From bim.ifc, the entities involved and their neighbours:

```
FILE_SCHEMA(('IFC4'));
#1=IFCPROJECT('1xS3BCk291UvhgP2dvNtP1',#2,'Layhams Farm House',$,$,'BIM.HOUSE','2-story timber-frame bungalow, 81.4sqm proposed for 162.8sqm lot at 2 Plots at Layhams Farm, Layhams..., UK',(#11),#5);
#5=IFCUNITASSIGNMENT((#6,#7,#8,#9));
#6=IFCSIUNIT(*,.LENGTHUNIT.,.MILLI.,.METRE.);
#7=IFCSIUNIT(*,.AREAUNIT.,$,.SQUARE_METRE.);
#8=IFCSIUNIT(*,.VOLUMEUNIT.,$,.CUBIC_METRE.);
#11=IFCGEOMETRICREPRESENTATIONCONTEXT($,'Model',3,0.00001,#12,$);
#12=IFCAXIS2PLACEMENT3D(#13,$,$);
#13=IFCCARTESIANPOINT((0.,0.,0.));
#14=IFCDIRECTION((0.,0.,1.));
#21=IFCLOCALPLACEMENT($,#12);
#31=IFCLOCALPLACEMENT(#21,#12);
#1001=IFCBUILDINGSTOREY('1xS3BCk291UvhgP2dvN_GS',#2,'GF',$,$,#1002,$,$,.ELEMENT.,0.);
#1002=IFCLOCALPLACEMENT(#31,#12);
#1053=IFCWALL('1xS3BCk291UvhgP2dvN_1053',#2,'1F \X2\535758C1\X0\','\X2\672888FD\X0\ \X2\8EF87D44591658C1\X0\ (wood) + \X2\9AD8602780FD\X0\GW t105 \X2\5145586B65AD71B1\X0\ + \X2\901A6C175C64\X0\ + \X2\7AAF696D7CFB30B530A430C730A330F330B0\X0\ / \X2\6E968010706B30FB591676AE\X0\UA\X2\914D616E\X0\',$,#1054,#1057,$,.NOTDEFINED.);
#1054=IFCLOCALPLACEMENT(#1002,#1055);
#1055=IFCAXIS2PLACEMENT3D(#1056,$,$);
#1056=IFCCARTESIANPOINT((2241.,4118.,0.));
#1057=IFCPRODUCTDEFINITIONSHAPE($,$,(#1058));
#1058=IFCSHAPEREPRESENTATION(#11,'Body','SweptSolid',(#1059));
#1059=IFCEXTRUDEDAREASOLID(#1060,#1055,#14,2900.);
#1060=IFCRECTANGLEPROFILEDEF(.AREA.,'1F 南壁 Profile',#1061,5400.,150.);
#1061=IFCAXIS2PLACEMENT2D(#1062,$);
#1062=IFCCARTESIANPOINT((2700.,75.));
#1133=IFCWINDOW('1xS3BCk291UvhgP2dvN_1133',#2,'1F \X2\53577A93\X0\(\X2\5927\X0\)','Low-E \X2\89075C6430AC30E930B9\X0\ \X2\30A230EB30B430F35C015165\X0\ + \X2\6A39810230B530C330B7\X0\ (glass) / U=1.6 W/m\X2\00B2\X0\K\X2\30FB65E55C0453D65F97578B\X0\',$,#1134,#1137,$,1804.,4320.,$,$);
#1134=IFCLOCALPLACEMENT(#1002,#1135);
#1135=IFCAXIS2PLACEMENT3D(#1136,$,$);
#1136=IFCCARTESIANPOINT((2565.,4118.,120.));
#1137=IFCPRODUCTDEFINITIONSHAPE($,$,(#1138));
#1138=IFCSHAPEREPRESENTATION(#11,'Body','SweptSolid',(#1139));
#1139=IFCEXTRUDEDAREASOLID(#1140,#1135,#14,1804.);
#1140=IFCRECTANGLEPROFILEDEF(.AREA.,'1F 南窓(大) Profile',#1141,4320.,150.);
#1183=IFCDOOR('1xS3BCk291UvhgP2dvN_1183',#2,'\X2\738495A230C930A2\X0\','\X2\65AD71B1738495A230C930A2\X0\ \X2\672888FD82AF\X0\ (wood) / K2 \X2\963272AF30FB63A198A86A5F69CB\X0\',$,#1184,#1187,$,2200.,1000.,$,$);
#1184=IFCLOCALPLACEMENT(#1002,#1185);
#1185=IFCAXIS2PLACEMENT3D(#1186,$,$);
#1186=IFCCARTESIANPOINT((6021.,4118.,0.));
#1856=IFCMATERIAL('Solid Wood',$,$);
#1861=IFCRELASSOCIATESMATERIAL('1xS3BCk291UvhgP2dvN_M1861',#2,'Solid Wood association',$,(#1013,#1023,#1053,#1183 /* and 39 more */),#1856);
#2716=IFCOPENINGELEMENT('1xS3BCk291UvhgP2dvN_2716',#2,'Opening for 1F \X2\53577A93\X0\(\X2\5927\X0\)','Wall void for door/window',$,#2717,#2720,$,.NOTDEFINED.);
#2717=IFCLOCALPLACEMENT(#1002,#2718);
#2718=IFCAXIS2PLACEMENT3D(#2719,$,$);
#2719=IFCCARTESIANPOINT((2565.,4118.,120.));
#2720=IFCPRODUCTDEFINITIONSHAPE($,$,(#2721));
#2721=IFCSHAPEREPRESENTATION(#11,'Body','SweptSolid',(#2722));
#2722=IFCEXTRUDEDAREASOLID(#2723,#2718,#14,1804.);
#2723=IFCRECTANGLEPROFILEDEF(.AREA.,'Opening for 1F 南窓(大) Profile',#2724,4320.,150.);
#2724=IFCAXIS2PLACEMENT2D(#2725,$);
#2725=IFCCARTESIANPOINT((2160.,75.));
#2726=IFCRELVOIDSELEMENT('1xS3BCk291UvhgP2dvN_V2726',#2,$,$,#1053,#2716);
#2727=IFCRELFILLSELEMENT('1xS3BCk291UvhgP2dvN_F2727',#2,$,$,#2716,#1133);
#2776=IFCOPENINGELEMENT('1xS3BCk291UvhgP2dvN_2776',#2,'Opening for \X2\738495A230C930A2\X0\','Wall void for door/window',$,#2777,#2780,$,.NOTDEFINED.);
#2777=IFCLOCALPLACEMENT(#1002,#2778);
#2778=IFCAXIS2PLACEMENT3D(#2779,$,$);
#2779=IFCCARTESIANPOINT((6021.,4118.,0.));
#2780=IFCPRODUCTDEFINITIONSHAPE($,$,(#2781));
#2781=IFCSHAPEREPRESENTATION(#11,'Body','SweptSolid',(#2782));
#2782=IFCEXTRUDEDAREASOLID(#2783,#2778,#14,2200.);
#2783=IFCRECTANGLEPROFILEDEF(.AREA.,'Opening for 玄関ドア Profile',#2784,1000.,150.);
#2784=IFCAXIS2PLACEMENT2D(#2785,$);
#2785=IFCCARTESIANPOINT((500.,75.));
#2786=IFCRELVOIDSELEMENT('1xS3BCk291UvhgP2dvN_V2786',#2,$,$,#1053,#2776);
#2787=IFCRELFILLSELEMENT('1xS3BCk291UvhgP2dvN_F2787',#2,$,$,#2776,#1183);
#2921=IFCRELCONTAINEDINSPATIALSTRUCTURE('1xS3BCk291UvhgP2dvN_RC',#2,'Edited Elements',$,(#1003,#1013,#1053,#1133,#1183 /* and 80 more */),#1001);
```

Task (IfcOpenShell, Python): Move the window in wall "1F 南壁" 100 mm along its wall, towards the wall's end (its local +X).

```python
import ifcopenshell
import ifcopenshell.api.geometry
import ifcopenshell.util.placement

model = ifcopenshell.open("bim.ifc")

window = model.by_guid("1xS3BCk291UvhgP2dvN_1133")
opening = window.FillsVoids[0].RelatingOpeningElement
wall = opening.VoidsElements[0].RelatingBuildingElement

wall_matrix = ifcopenshell.util.placement.get_local_placement(wall.ObjectPlacement)
shift = wall_matrix[:3, 0] * 100.0
before = ifcopenshell.util.placement.get_local_placement(window.ObjectPlacement)[:3, 3].copy()

# The window is not placed relative to its opening, so move both.
for product in (opening, window):
    matrix = ifcopenshell.util.placement.get_local_placement(product.ObjectPlacement)
    matrix[:3, 3] += shift
    ifcopenshell.api.geometry.edit_object_placement(model, product=product, matrix=matrix, is_si=False)

after = ifcopenshell.util.placement.get_local_placement(window.ObjectPlacement)[:3, 3]
print("window moved by", (after - before).round(3) + 0.0)

model.write("bim_updated.ifc")
```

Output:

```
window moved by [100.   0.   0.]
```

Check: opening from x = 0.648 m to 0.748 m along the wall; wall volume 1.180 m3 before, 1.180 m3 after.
